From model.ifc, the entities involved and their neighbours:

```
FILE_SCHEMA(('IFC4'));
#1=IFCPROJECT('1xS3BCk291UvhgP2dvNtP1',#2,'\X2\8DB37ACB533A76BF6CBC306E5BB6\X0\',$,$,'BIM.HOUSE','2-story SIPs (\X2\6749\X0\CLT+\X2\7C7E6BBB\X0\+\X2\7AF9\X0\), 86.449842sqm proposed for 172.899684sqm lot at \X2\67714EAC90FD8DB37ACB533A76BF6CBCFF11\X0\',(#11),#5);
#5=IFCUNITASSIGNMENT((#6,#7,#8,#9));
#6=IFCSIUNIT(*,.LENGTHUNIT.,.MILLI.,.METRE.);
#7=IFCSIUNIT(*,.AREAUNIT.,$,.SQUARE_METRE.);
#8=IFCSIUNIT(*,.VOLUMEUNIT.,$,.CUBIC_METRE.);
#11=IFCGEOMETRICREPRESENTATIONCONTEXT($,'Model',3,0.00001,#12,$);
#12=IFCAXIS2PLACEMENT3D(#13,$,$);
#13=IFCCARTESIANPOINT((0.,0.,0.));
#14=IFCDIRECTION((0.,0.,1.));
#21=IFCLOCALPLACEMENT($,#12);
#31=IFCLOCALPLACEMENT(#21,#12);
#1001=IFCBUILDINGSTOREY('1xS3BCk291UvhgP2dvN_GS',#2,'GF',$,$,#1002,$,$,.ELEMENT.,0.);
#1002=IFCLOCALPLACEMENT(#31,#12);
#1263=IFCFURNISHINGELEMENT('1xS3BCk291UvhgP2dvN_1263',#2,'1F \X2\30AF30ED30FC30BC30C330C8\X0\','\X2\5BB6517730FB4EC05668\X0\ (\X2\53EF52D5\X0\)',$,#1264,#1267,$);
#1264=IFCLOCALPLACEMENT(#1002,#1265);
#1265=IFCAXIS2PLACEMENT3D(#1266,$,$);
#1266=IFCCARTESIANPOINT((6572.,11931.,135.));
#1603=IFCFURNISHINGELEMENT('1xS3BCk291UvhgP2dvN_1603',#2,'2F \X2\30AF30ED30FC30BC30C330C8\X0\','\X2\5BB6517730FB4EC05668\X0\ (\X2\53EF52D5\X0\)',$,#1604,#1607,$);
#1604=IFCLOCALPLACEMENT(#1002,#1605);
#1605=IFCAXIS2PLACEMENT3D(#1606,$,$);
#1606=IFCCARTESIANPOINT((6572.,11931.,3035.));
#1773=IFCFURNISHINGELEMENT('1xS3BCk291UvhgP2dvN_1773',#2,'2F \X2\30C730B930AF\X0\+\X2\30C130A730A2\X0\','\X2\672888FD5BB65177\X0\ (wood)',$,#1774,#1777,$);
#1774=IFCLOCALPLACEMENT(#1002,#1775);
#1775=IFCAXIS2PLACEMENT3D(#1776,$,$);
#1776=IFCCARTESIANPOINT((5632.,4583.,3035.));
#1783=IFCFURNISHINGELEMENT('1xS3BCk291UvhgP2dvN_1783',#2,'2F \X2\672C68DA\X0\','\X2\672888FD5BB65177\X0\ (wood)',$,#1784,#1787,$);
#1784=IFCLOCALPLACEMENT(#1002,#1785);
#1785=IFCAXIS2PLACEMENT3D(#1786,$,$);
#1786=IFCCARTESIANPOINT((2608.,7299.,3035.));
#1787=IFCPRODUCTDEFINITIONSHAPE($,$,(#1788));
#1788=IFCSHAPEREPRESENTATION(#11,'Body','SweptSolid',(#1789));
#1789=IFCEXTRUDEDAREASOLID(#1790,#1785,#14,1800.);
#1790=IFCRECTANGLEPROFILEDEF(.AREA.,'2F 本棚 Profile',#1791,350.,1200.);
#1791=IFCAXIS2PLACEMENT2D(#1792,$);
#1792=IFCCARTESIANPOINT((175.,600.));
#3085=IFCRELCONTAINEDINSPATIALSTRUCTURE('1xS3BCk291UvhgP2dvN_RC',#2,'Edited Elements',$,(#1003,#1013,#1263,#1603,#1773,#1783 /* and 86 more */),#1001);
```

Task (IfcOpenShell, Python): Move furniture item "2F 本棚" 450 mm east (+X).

```python
import ifcopenshell
import ifcopenshell.api.geometry
import ifcopenshell.util.placement
import ifcopenshell.util.unit

model = ifcopenshell.open("model.ifc")
unit_scale = ifcopenshell.util.unit.calculate_unit_scale(model)

item = model.by_id(1783)
matrix = ifcopenshell.util.placement.get_local_placement(item.ObjectPlacement)
matrix[0, 3] += 0.45 / unit_scale
ifcopenshell.api.geometry.edit_object_placement(model, product=item, matrix=matrix, is_si=False)

print(ifcopenshell.util.placement.get_local_placement(item.ObjectPlacement).round(3) + 0.0)

model.write("model_updated.ifc")
```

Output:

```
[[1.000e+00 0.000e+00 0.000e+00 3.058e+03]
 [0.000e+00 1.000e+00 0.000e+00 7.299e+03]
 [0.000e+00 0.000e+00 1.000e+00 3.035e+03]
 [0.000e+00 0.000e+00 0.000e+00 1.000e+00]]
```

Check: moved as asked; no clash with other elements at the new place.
